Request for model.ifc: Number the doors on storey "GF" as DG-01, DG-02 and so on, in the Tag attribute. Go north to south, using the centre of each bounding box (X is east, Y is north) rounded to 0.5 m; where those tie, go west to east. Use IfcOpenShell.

First a look at what the model holds.

```python
import ifcopenshell
import ifcopenshell.util.element
import ifcopenshell.util.placement

model = ifcopenshell.open("model.ifc")
print(model.schema)
storey = next(s for s in model.by_type("IfcBuildingStorey") if s.Name == "GF")
doors = [e for e in ifcopenshell.util.element.get_decomposition(storey) if e.is_a("IfcDoor")]
for e in sorted(doors, key=lambda e: e.id()):
    origin = ifcopenshell.util.placement.get_local_placement(e.ObjectPlacement)[:3, 3]
    print(e.id(), e.Tag, e.Name, origin.round(2) + 0.0, sep=" | ")
```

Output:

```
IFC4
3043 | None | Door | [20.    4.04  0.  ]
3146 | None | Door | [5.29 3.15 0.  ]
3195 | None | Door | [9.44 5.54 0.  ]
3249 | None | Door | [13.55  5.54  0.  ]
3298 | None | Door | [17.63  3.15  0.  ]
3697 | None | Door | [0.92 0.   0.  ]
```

```python
import ifcopenshell
import ifcopenshell.geom
import ifcopenshell.util.element
import ifcopenshell.util.shape

model = ifcopenshell.open("model.ifc")
settings = ifcopenshell.geom.settings()
settings.set("use-world-coords", True)


def centre(element):
    shape = ifcopenshell.geom.create_shape(settings, element)
    return ifcopenshell.util.shape.get_bbox_centroid(shape.geometry)


storey = next(s for s in model.by_type("IfcBuildingStorey") if s.Name == "GF")
doors = [e for e in ifcopenshell.util.element.get_decomposition(storey) if e.is_a("IfcDoor")]

# Insertion points can sit at a corner or the storey origin, so sort by the geometry (in metres).
centres = {e: centre(e) for e in doors}
doors.sort(key=lambda e: (-round(centres[e][1] / 0.5), centres[e][0]))

for i, e in enumerate(doors, start=1):
    number = f"DG-{i:02d}"
    e.Tag = number
    print(e.id(), number)

model.write("model_edited.ifc")
```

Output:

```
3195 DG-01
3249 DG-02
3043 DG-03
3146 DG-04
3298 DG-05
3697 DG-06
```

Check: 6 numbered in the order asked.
